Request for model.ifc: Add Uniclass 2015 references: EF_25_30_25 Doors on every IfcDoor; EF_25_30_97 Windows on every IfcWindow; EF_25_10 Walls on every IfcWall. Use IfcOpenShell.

First a look at what the model holds.

```python
import ifcopenshell

model = ifcopenshell.open("model.ifc")
print(model.schema)
print("classifications:", [c.Name for c in model.by_type("IfcClassification")])
for ifc_class in ("IfcDoor", "IfcRoof", "IfcStair", "IfcWall", "IfcWindow"):
    print(ifc_class, len(model.by_type(ifc_class)))
```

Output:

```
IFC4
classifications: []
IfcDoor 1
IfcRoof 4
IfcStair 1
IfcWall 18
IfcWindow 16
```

```python
import ifcopenshell
import ifcopenshell.api.classification

model = ifcopenshell.open("model.ifc")

system = ifcopenshell.api.classification.add_classification(model, classification="Uniclass 2015")

codes = {
    "IfcDoor": ("EF_25_30_25", "Doors"),
    "IfcWindow": ("EF_25_30_97", "Windows"),
    "IfcWall": ("EF_25_10", "Walls"),
}
for ifc_class, (code, name) in codes.items():
    products = model.by_type(ifc_class)
    ifcopenshell.api.classification.add_reference(
        model, products=products, classification=system, identification=code, name=name
    )
    print(code, len(products))

model.write("model_edited.ifc")
```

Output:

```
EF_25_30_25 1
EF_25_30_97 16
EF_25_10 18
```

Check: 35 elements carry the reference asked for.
